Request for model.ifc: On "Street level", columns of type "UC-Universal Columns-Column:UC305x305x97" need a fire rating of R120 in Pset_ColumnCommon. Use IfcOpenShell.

First a look at what the model holds.

```python
import ifcopenshell
import ifcopenshell.util.element

model = ifcopenshell.open("model.ifc")
print(model.schema)
storey = next(s for s in model.by_type("IfcBuildingStorey") if s.Name == "Street level")
columns = [e for e in ifcopenshell.util.element.get_decomposition(storey) if e.is_a("IfcColumn")]
seen = {}
for e in columns:
    element_type = ifcopenshell.util.element.get_type(e)
    key = (element_type.Name if element_type != e and element_type else None, ifcopenshell.util.element.get_pset(e, "Pset_ColumnCommon", "FireRating"))
    seen[key] = seen.get(key, 0) + 1
for (name, value), count in sorted(seen.items(), key=str):
    print(count, "x", name, "|", value)
```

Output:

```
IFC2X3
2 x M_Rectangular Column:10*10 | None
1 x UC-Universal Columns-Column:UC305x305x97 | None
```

```python
import ifcopenshell
import ifcopenshell.api.pset
import ifcopenshell.util.element

model = ifcopenshell.open("model.ifc")

storey = next(s for s in model.by_type("IfcBuildingStorey") if s.Name == "Street level")
columns = [e for e in ifcopenshell.util.element.get_decomposition(storey) if e.is_a("IfcColumn")]

count = 0
for e in columns:
    element_type = ifcopenshell.util.element.get_type(e)
    if element_type in (None, e) or element_type.Name != "UC-Universal Columns-Column:UC305x305x97":
        continue
    # add_pset returns the element's existing set when there is one.
    pset = ifcopenshell.api.pset.add_pset(model, product=e, name="Pset_ColumnCommon")
    ifcopenshell.api.pset.edit_pset(model, pset=pset, properties={"FireRating": "R120"})
    count += 1

print(count, "columns updated")

model.write("model_edited.ifc")
```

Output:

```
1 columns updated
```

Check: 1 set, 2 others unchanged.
